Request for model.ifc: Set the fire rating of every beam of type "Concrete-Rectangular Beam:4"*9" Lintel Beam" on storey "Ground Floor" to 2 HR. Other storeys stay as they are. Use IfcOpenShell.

First a look at what the model holds.

```python
import ifcopenshell
import ifcopenshell.util.element

model = ifcopenshell.open("model.ifc")
print(model.schema)
storey = next(s for s in model.by_type("IfcBuildingStorey") if s.Name == "Ground Floor")
beams = [e for e in ifcopenshell.util.element.get_decomposition(storey) if e.is_a("IfcBeam")]
seen = {}
for e in beams:
    element_type = ifcopenshell.util.element.get_type(e)
    key = (element_type.Name if element_type != e and element_type else None, ifcopenshell.util.element.get_pset(e, "Pset_BeamCommon", "FireRating"))
    seen[key] = seen.get(key, 0) + 1
for (name, value), count in sorted(seen.items(), key=str):
    print(count, "x", name, "|", value)
```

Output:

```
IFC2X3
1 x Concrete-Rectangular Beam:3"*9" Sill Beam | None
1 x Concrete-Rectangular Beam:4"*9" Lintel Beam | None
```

```python
import ifcopenshell
import ifcopenshell.api.pset
import ifcopenshell.util.element

model = ifcopenshell.open("model.ifc")

storey = next(s for s in model.by_type("IfcBuildingStorey") if s.Name == "Ground Floor")
beams = [e for e in ifcopenshell.util.element.get_decomposition(storey) if e.is_a("IfcBeam")]

count = 0
for e in beams:
    element_type = ifcopenshell.util.element.get_type(e)
    if element_type in (None, e) or element_type.Name != 'Concrete-Rectangular Beam:4"*9" Lintel Beam':
        continue
    # add_pset returns the element's existing set when there is one.
    pset = ifcopenshell.api.pset.add_pset(model, product=e, name="Pset_BeamCommon")
    ifcopenshell.api.pset.edit_pset(model, pset=pset, properties={"FireRating": "2 HR"})
    count += 1

print(count, "beams updated")

model.write("model_v2.ifc")
```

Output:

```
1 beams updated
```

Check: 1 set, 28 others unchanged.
